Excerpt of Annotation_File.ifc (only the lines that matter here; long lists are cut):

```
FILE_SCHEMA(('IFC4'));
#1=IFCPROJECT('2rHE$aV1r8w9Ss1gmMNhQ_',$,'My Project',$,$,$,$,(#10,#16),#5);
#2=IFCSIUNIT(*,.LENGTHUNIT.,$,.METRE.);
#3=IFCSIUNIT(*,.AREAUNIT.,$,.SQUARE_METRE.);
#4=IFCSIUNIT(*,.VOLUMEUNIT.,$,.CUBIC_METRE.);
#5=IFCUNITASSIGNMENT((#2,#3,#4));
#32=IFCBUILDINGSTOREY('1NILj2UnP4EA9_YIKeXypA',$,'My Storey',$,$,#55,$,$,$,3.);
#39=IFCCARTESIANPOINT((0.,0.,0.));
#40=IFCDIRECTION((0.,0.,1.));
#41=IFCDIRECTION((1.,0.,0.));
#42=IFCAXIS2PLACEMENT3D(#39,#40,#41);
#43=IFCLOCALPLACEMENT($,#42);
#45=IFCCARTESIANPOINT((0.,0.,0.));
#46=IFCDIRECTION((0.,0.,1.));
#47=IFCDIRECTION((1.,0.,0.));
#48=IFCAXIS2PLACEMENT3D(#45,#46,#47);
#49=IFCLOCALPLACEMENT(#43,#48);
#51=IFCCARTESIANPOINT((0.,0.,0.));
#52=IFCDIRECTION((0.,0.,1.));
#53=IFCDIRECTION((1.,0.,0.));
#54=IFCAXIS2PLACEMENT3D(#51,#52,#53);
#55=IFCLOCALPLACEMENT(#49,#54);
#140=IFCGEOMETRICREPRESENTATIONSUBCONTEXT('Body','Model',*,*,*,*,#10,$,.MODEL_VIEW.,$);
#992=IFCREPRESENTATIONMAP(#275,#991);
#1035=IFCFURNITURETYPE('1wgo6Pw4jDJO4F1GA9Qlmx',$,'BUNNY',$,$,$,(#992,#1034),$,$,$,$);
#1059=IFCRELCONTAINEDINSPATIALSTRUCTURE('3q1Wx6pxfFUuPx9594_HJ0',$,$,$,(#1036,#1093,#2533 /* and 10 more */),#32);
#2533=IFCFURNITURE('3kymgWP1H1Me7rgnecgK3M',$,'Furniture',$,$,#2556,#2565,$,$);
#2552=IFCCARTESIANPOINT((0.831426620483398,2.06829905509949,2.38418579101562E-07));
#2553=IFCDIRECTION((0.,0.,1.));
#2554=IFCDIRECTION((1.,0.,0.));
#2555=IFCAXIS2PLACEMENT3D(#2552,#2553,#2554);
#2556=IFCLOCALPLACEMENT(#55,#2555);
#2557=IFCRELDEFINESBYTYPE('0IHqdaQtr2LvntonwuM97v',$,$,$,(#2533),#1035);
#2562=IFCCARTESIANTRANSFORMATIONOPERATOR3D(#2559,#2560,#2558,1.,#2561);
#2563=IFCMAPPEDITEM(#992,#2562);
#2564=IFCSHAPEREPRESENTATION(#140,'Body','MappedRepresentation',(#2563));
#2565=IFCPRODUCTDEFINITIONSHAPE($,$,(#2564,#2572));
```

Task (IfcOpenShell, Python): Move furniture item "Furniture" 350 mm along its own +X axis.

```python
import ifcopenshell
import ifcopenshell.api.geometry
import ifcopenshell.util.placement

model = ifcopenshell.open("Annotation_File.ifc")

item = model.by_guid("3kymgWP1H1Me7rgnecgK3M")
matrix = ifcopenshell.util.placement.get_local_placement(item.ObjectPlacement)
matrix[:3, 3] += matrix[:3, 0] * 0.35
ifcopenshell.api.geometry.edit_object_placement(model, product=item, matrix=matrix, is_si=False)

print(ifcopenshell.util.placement.get_local_placement(item.ObjectPlacement).round(3) + 0.0)

model.write("Annotation_File_rev.ifc")
```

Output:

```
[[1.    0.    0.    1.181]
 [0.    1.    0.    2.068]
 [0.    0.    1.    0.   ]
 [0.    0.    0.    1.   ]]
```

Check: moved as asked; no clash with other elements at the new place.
